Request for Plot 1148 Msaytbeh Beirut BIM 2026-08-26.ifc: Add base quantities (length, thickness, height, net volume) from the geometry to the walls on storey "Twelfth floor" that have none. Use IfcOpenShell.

First a look at what the model holds.

```python
import ifcopenshell
import ifcopenshell.util.element
import ifcopenshell.util.unit

model = ifcopenshell.open("Plot 1148 Msaytbeh Beirut BIM 2026-08-26.ifc")
print(model.schema)
for unit_type in ("LENGTHUNIT", "AREAUNIT", "VOLUMEUNIT"):
    print(unit_type, ifcopenshell.util.unit.calculate_unit_scale(model, unit_type))
storey = next(s for s in model.by_type("IfcBuildingStorey") if s.Name == "Twelfth floor")
walls = [e for e in ifcopenshell.util.element.get_decomposition(storey) if e.is_a("IfcWall")]
for e in sorted(walls, key=lambda e: e.id()):
    print(e.id(), e.is_a(), e.Name, list(ifcopenshell.util.element.get_psets(e, qtos_only=True)), sep=" | ")
```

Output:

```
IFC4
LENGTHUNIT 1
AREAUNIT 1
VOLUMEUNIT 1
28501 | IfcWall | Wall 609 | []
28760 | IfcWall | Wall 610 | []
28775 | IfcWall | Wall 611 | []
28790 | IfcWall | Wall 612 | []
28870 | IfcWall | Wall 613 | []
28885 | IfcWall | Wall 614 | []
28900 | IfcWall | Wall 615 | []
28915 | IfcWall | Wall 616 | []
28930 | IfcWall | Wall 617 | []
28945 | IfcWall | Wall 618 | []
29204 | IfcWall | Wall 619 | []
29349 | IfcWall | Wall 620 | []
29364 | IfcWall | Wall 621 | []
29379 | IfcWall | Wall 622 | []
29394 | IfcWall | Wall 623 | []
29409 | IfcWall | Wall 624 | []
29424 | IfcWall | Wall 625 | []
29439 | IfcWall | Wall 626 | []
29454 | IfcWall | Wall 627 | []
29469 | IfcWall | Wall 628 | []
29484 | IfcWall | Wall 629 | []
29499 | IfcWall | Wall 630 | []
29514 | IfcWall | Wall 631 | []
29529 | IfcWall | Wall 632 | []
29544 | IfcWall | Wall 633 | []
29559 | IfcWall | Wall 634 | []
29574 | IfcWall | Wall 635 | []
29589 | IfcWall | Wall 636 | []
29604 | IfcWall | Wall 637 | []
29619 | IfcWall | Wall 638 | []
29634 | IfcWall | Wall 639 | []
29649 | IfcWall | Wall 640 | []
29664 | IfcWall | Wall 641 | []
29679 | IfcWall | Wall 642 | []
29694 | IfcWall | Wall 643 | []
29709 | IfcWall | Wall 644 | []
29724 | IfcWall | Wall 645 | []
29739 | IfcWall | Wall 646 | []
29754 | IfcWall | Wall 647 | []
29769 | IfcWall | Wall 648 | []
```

```python
import ifcopenshell
import ifcopenshell.api.pset
import ifcopenshell.geom
import ifcopenshell.util.element
import ifcopenshell.util.shape
import ifcopenshell.util.unit

model = ifcopenshell.open("Plot 1148 Msaytbeh Beirut BIM 2026-08-26.ifc")
unit_scale = ifcopenshell.util.unit.calculate_unit_scale(model)
volume_scale = ifcopenshell.util.unit.calculate_unit_scale(model, "VOLUMEUNIT")
settings = ifcopenshell.geom.settings()

storey = next(s for s in model.by_type("IfcBuildingStorey") if s.Name == "Twelfth floor")
walls = [e for e in ifcopenshell.util.element.get_decomposition(storey) if e.is_a("IfcWall")]

for e in sorted(walls, key=lambda e: e.id()):
    if ifcopenshell.util.element.get_psets(e, qtos_only=True, should_inherit=False):
        continue
    # Geometry comes back in metres, in the element's own axes.
    shape = ifcopenshell.geom.create_shape(settings, e)
    values = {
        "Length": ifcopenshell.util.shape.get_x(shape.geometry) / unit_scale,
        "Width": ifcopenshell.util.shape.get_y(shape.geometry) / unit_scale,
        "Height": ifcopenshell.util.shape.get_z(shape.geometry) / unit_scale,
        "NetVolume": ifcopenshell.util.shape.get_volume(shape.geometry) / volume_scale,
    }
    qto = ifcopenshell.api.pset.add_qto(model, product=e, name="Qto_WallBaseQuantities")
    ifcopenshell.api.pset.edit_qto(model, qto=qto, properties=values)
    print(e.id(), {k: round(v, 3) for k, v in values.items()})

model.write("Plot 1148 Msaytbeh Beirut BIM 2026-08-26_v2.ifc")
```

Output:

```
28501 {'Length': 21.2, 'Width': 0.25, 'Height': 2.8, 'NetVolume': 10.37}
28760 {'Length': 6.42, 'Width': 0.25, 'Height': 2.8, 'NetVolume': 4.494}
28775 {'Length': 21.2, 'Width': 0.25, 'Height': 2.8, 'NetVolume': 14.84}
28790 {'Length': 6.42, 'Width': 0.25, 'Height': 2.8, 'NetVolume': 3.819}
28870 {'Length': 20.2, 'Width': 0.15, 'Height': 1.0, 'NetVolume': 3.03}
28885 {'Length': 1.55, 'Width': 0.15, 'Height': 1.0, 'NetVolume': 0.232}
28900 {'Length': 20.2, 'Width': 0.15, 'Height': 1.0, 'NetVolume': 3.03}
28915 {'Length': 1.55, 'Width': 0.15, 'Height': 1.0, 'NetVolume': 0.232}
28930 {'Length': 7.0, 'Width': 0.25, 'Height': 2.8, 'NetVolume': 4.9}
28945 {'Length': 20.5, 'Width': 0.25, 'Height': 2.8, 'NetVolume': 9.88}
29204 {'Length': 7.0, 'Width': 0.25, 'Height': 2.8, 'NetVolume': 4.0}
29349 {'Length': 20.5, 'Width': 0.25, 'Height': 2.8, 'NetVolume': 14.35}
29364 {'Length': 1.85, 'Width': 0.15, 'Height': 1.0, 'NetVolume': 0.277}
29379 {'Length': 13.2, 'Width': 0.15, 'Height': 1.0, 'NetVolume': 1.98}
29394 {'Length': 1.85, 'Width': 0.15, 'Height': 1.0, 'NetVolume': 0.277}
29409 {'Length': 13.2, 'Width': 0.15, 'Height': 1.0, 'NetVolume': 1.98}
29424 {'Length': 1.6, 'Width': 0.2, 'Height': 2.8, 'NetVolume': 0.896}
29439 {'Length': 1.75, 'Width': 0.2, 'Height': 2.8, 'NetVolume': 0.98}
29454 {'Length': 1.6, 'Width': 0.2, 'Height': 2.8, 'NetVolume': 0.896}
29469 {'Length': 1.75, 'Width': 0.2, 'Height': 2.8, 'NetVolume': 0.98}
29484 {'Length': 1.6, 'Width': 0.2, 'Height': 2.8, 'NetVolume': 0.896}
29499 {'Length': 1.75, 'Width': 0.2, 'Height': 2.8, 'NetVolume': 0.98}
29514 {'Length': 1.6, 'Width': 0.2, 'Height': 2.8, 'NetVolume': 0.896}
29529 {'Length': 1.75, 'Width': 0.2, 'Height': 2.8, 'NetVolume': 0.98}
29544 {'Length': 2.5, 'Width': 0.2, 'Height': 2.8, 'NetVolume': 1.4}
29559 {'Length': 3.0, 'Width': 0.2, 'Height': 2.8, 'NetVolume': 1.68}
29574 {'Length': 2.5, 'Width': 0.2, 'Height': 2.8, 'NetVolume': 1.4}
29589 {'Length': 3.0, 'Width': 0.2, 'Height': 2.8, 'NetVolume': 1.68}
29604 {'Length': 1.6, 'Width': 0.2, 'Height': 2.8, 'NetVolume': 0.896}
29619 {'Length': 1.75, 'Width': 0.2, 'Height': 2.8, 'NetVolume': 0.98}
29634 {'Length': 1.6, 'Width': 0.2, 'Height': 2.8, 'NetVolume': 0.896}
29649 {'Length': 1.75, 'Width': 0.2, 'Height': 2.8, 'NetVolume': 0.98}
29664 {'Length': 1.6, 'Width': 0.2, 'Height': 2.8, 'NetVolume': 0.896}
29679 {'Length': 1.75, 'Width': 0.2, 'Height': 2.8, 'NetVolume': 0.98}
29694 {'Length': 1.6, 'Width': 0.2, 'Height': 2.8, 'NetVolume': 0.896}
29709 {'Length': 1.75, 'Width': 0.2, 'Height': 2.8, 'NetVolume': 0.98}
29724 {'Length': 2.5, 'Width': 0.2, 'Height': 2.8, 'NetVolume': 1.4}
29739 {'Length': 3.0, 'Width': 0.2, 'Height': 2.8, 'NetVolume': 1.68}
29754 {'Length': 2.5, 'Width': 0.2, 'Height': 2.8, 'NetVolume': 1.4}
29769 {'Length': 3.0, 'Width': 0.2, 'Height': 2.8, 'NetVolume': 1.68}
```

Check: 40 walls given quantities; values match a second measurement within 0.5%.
